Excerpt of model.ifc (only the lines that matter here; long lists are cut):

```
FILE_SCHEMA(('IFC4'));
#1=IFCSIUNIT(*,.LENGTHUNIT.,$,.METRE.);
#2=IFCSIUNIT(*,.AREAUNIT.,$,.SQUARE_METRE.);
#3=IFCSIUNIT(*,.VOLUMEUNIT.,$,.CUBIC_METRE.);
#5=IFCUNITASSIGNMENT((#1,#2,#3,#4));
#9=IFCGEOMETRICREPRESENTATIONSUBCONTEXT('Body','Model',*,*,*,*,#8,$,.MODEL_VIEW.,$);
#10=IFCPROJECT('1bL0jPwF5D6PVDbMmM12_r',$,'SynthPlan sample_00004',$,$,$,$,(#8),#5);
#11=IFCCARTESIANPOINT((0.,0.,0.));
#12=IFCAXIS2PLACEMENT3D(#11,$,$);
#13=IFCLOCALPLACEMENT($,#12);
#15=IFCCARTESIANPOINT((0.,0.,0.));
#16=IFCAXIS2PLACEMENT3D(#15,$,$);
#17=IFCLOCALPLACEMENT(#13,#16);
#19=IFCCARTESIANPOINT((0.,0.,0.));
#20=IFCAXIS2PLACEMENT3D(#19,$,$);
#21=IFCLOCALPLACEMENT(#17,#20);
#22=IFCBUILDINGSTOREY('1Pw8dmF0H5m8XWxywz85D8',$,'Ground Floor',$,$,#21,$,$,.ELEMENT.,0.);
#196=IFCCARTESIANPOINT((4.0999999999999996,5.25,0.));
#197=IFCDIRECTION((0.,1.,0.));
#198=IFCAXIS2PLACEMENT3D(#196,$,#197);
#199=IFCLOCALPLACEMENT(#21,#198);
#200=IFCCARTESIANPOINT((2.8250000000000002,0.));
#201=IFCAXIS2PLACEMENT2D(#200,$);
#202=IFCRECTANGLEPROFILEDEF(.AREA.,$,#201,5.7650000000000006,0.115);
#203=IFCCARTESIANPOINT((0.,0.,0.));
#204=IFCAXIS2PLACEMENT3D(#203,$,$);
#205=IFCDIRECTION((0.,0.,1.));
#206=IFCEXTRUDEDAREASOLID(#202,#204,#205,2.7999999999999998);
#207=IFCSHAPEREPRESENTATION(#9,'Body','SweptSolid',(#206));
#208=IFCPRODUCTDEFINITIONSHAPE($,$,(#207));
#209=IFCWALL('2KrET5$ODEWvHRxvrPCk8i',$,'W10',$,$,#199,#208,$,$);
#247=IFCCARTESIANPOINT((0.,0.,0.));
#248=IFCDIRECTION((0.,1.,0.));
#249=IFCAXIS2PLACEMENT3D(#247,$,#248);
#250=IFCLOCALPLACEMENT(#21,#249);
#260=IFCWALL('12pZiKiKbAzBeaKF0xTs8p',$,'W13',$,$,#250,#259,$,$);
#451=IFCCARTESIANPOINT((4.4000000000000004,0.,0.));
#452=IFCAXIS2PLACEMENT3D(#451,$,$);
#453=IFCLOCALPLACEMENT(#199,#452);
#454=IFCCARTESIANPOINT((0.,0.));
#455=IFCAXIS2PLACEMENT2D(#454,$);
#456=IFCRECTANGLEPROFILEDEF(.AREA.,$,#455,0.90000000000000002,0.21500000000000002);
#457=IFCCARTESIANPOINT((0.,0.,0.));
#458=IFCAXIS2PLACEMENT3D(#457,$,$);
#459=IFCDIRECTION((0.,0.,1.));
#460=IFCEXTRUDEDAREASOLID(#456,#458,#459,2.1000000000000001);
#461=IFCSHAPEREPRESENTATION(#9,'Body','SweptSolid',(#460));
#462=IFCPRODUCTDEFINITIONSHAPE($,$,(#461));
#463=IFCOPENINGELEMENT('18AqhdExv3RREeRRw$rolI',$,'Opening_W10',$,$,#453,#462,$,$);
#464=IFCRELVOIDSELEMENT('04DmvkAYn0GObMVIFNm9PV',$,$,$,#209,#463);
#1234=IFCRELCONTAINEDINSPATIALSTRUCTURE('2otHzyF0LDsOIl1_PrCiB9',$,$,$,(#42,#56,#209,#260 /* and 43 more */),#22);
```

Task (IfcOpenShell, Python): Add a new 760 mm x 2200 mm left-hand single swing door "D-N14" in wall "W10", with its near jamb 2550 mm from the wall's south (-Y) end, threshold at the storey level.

```python
import numpy as np
import ifcopenshell
import ifcopenshell.api.feature
import ifcopenshell.api.geometry
import ifcopenshell.api.root
import ifcopenshell.api.spatial
import ifcopenshell.geom
import ifcopenshell.util.element
import ifcopenshell.util.placement
import ifcopenshell.util.representation
import ifcopenshell.util.shape
import ifcopenshell.util.unit

model = ifcopenshell.open("model.ifc")
unit_scale = ifcopenshell.util.unit.calculate_unit_scale(model)
settings = ifcopenshell.geom.settings()


def volume(element):
    """Net volume in cubic metres, openings subtracted."""
    shape = ifcopenshell.geom.create_shape(settings, element)
    return ifcopenshell.util.shape.get_volume(shape.geometry)


wall = model.by_id(209)
storey = ifcopenshell.util.element.get_container(wall, ifc_class="IfcBuildingStorey")
context = ifcopenshell.util.representation.get_context(model, "Model", "Body", "MODEL_VIEW")
before = volume(wall)

width, height, from_end, sill = 0.76, 2.2, 2.55, 0.0  # metres

# The wall runs along its own X axis, and the end named is its -X end.
wall_shape = ifcopenshell.geom.create_shape(settings, wall)
x, y, z = ifcopenshell.util.shape.get_vertices(wall_shape.geometry).T
start = x.min() + from_end
face, thickness = float(y.min()), float(y.max() - y.min())
wall_matrix = ifcopenshell.util.placement.get_local_placement(wall.ObjectPlacement)
level = ifcopenshell.util.placement.get_local_placement(storey.ObjectPlacement)[2, 3]


def in_wall(x, y):
    """Placement at x, y metres in the wall's axes, at sill height."""
    matrix = wall_matrix.copy()
    matrix[:, 3] = wall_matrix @ np.array([x / unit_scale, y / unit_scale, 0.0, 1.0])
    matrix[2, 3] = level + sill / unit_scale
    return matrix


# Opening: a box that overshoots both wall faces by 50 mm.
opening = ifcopenshell.api.root.create_entity(model, ifc_class="IfcOpeningElement", predefined_type="OPENING")
box = ifcopenshell.api.geometry.add_wall_representation(
    model, context=context, length=width, height=height, thickness=thickness + 0.1
)
ifcopenshell.api.geometry.assign_representation(model, product=opening, representation=box)
ifcopenshell.api.geometry.edit_object_placement(model, product=opening, matrix=in_wall(start, face - 0.05), is_si=False)
ifcopenshell.api.feature.add_feature(model, feature=opening, element=wall)

door = ifcopenshell.api.root.create_entity(model, ifc_class="IfcDoor", name="D-N14", predefined_type="DOOR")
door.OverallWidth, door.OverallHeight = width / unit_scale, height / unit_scale
door.OperationType = "SINGLE_SWING_LEFT"
body = ifcopenshell.api.geometry.add_door_representation(
    model,
    context=context,
    overall_width=door.OverallWidth,
    overall_height=door.OverallHeight,
    operation_type="SINGLE_SWING_LEFT",
    lining_properties={"LiningDepth": thickness / unit_scale, "ThresholdDepth": thickness / unit_scale},
)
ifcopenshell.api.geometry.assign_representation(model, product=door, representation=body)
ifcopenshell.api.spatial.assign_container(model, products=[door], relating_structure=storey)
ifcopenshell.api.feature.add_filling(model, opening=opening, element=door)

# The lining spans the wall, so the door starts at the wall face.
ifcopenshell.api.geometry.edit_object_placement(model, product=door, matrix=in_wall(start, face), is_si=False)

after = volume(wall)

print(f"wall volume {before:.3f} -> {after:.3f} m3")

model.write("model_rev.ifc")
```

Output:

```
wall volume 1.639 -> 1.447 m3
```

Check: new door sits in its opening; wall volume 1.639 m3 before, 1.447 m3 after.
